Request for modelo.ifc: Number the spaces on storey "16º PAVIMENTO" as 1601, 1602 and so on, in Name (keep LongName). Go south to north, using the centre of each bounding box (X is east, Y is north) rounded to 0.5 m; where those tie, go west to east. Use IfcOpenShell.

First a look at what the model holds.

```python
import ifcopenshell
import ifcopenshell.util.element
import ifcopenshell.util.placement

model = ifcopenshell.open("modelo.ifc")
print(model.schema)
storey = next(s for s in model.by_type("IfcBuildingStorey") if s.Name == "16º PAVIMENTO")
spaces = [e for e in ifcopenshell.util.element.get_decomposition(storey) if e.is_a("IfcSpace")]
for e in sorted(spaces, key=lambda e: e.id()):
    origin = ifcopenshell.util.placement.get_local_placement(e.ObjectPlacement)[:3, 3]
    print(e.id(), e.Name, e.LongName, origin.round(2) + 0.0, sep=" | ")
```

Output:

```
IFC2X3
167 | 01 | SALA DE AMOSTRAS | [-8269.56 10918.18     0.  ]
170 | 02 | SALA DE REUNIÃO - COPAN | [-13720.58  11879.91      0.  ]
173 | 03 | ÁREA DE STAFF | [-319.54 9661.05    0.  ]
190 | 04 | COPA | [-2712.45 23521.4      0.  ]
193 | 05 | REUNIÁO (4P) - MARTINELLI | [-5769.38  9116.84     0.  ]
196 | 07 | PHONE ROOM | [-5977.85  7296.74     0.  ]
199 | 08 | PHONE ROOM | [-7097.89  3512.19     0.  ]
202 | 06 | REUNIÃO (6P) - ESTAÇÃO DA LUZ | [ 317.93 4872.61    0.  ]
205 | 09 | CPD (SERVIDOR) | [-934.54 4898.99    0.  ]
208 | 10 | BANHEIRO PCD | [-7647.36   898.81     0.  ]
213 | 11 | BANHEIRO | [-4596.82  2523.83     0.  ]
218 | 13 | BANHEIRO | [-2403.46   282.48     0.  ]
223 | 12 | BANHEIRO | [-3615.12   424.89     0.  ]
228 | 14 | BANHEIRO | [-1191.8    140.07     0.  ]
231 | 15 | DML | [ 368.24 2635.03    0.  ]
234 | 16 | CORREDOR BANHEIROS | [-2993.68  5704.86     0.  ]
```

```python
import ifcopenshell
import ifcopenshell.geom
import ifcopenshell.util.element
import ifcopenshell.util.shape

model = ifcopenshell.open("modelo.ifc")
settings = ifcopenshell.geom.settings()
settings.set("use-world-coords", True)


def centre(element):
    shape = ifcopenshell.geom.create_shape(settings, element)
    return ifcopenshell.util.shape.get_bbox_centroid(shape.geometry)


storey = next(s for s in model.by_type("IfcBuildingStorey") if s.Name == "16º PAVIMENTO")
spaces = [e for e in ifcopenshell.util.element.get_decomposition(storey) if e.is_a("IfcSpace")]

# Insertion points can sit at a corner or the storey origin, so sort by the geometry (in metres).
centres = {e: centre(e) for e in spaces}
spaces.sort(key=lambda e: (round(centres[e][1] / 0.5), centres[e][0]))

for i, e in enumerate(spaces, start=1):
    number = f"16{i:02d}"
    e.Name = number
    print(e.id(), number)

model.write("modelo_updated.ifc")
```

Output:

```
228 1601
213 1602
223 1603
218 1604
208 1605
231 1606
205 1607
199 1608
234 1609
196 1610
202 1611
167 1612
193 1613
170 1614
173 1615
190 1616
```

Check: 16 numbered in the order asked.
